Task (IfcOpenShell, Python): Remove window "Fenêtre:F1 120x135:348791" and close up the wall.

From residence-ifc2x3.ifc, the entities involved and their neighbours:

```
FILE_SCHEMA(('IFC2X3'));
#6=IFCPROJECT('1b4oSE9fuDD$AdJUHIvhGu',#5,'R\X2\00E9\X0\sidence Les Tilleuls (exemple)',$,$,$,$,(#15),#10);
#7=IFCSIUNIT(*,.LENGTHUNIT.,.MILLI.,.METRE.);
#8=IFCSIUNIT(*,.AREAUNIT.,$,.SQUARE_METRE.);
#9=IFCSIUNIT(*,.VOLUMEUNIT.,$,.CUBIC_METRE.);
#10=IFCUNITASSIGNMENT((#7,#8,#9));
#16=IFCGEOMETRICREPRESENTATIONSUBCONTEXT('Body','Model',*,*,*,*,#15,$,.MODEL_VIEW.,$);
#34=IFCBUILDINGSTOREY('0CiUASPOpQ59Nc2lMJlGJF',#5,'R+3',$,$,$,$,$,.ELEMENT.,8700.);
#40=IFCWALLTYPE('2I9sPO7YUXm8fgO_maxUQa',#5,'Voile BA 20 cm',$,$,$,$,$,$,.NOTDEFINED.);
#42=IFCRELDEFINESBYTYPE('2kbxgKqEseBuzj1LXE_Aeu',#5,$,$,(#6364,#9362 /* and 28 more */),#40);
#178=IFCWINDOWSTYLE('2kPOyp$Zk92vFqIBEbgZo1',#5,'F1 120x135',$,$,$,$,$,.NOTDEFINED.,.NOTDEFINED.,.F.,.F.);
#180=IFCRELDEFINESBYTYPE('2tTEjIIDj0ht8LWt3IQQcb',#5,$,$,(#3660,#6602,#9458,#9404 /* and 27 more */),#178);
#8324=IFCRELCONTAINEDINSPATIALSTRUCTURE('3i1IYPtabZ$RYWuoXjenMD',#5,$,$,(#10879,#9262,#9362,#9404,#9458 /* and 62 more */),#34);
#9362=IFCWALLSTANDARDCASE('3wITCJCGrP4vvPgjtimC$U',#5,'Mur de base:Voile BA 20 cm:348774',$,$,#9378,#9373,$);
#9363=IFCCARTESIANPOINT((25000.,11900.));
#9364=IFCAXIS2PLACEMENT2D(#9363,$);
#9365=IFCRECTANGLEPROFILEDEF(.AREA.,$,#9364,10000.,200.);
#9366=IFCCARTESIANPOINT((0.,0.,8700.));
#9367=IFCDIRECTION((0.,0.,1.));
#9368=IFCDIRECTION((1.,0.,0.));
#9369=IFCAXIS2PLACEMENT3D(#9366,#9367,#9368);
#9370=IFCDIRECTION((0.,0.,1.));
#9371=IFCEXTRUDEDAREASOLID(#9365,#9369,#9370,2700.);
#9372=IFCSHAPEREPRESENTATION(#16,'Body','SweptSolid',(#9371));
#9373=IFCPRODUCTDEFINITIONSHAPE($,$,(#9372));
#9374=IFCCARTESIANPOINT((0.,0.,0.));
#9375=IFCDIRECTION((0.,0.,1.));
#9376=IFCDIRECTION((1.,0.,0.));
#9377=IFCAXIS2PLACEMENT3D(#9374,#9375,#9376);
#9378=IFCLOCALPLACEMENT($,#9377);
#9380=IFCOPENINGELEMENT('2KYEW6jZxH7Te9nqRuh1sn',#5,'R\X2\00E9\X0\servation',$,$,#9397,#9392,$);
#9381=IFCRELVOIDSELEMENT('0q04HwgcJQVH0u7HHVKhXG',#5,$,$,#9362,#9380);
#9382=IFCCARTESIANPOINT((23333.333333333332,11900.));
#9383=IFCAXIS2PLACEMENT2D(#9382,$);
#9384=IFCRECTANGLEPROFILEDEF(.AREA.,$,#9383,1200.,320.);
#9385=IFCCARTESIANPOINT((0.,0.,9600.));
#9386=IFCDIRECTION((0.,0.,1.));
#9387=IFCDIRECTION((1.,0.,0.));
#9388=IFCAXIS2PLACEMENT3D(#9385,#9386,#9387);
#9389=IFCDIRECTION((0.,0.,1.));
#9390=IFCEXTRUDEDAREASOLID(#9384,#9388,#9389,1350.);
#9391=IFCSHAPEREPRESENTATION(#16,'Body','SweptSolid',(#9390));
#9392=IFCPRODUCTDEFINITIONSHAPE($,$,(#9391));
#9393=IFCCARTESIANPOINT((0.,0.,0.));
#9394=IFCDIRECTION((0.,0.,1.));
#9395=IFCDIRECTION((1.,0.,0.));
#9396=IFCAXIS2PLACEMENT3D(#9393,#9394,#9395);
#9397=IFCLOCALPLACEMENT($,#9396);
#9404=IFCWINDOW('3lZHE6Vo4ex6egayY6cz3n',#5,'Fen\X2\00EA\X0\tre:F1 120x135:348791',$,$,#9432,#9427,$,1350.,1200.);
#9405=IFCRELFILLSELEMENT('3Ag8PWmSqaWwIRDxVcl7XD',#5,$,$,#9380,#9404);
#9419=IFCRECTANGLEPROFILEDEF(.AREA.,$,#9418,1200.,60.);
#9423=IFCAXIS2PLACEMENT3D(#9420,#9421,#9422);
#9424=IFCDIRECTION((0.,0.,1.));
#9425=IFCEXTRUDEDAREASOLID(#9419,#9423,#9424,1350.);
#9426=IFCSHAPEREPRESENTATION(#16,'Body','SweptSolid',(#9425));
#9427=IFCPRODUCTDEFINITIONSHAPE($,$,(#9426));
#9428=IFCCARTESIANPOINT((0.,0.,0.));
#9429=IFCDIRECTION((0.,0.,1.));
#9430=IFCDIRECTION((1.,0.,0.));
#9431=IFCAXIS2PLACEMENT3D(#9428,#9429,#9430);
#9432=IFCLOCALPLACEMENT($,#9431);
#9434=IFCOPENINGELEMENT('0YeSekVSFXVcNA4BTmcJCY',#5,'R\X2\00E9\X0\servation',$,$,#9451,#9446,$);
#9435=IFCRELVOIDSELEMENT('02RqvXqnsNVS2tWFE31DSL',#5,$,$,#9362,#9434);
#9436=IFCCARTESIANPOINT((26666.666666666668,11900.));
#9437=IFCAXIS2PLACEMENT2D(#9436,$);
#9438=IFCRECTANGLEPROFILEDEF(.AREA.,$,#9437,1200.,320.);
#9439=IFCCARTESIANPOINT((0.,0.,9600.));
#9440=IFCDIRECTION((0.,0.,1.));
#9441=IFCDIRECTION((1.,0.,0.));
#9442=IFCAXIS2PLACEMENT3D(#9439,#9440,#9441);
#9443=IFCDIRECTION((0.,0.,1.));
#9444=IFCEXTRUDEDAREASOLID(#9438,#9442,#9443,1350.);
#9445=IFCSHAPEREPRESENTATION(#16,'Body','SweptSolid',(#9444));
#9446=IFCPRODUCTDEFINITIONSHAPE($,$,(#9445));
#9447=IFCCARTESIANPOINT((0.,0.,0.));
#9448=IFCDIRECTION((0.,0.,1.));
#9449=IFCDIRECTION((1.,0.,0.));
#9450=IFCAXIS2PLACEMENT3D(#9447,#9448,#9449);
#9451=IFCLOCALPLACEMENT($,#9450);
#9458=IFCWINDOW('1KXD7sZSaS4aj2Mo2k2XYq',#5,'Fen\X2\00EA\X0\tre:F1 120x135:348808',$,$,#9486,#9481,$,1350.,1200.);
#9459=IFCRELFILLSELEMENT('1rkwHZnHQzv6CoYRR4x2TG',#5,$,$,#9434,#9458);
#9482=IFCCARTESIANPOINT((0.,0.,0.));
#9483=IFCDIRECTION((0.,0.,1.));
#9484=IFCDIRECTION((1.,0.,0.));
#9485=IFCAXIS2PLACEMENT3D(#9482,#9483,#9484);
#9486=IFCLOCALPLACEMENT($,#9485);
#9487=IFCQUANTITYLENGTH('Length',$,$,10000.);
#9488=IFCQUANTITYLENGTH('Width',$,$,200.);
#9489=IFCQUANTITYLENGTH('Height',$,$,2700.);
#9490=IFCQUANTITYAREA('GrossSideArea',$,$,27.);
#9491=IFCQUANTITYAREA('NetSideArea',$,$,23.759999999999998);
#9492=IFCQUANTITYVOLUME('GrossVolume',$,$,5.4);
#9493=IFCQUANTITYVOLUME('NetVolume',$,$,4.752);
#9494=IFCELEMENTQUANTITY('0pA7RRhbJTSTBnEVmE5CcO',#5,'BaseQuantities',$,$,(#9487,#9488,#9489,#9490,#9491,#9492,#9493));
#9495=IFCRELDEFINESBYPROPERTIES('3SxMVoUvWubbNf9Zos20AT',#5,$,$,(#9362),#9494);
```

```python
import ifcopenshell
import ifcopenshell.api.feature
import ifcopenshell.api.pset
import ifcopenshell.api.root
import ifcopenshell.geom
import ifcopenshell.util.element
import ifcopenshell.util.shape
import ifcopenshell.util.unit

model = ifcopenshell.open("residence-ifc2x3.ifc")
area_scale = ifcopenshell.util.unit.calculate_unit_scale(model, "AREAUNIT")
volume_scale = ifcopenshell.util.unit.calculate_unit_scale(model, "VOLUMEUNIT")
settings = ifcopenshell.geom.settings()


def volume(element):
    """Net volume in cubic metres, openings subtracted."""
    shape = ifcopenshell.geom.create_shape(settings, element)
    return ifcopenshell.util.shape.get_volume(shape.geometry)


window = model.by_guid("3lZHE6Vo4ex6egayY6cz3n")
opening = window.FillsVoids[0].RelatingOpeningElement
wall = opening.VoidsElements[0].RelatingBuildingElement
before = volume(wall)

ifcopenshell.api.root.remove_product(model, product=window)
ifcopenshell.api.feature.remove_feature(model, feature=opening)

after = volume(wall)
thickness = 0.2  # wall thickness in metres

# Update the wall's stored quantities.
qto = model.by_id(ifcopenshell.util.element.get_pset(wall, "BaseQuantities", should_inherit=False)["id"])
ifcopenshell.api.pset.edit_qto(model, qto=qto, properties={
    "NetSideArea": after / thickness / area_scale,
    "NetVolume": after / volume_scale,
})

print(f"wall volume {before:.3f} -> {after:.3f} m3")

model.write("residence-ifc2x3_v2.ifc")
```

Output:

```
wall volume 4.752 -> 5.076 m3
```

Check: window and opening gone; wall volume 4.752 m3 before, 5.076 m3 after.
